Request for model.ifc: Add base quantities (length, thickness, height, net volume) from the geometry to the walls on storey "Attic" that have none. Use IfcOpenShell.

First a look at what the model holds.

```python
import ifcopenshell
import ifcopenshell.util.element
import ifcopenshell.util.unit

model = ifcopenshell.open("model.ifc")
print(model.schema)
for unit_type in ("LENGTHUNIT", "AREAUNIT", "VOLUMEUNIT"):
    print(unit_type, ifcopenshell.util.unit.calculate_unit_scale(model, unit_type))
storey = next(s for s in model.by_type("IfcBuildingStorey") if s.Name == "Attic")
walls = [e for e in ifcopenshell.util.element.get_decomposition(storey) if e.is_a("IfcWall")]
for e in sorted(walls, key=lambda e: e.id()):
    print(e.id(), e.is_a(), e.Name, list(ifcopenshell.util.element.get_psets(e, qtos_only=True)), sep=" | ")
```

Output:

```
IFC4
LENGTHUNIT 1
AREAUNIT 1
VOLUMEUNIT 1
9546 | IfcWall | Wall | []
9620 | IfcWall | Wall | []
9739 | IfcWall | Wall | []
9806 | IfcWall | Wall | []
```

```python
import ifcopenshell
import ifcopenshell.api.pset
import ifcopenshell.geom
import ifcopenshell.util.element
import ifcopenshell.util.shape
import ifcopenshell.util.unit

model = ifcopenshell.open("model.ifc")
unit_scale = ifcopenshell.util.unit.calculate_unit_scale(model)
volume_scale = ifcopenshell.util.unit.calculate_unit_scale(model, "VOLUMEUNIT")
settings = ifcopenshell.geom.settings()

storey = next(s for s in model.by_type("IfcBuildingStorey") if s.Name == "Attic")
walls = [e for e in ifcopenshell.util.element.get_decomposition(storey) if e.is_a("IfcWall")]

for e in sorted(walls, key=lambda e: e.id()):
    if ifcopenshell.util.element.get_psets(e, qtos_only=True, should_inherit=False):
        continue
    # Geometry comes back in metres, in the element's own axes.
    shape = ifcopenshell.geom.create_shape(settings, e)
    values = {
        "Length": ifcopenshell.util.shape.get_x(shape.geometry) / unit_scale,
        "Width": ifcopenshell.util.shape.get_y(shape.geometry) / unit_scale,
        "Height": ifcopenshell.util.shape.get_z(shape.geometry) / unit_scale,
        "NetVolume": ifcopenshell.util.shape.get_volume(shape.geometry) / volume_scale,
    }
    qto = ifcopenshell.api.pset.add_qto(model, product=e, name="Qto_WallBaseQuantities")
    ifcopenshell.api.pset.edit_qto(model, qto=qto, properties=values)
    print(e.id(), {k: round(v, 3) for k, v in values.items()})

model.write("model-out.ifc")
```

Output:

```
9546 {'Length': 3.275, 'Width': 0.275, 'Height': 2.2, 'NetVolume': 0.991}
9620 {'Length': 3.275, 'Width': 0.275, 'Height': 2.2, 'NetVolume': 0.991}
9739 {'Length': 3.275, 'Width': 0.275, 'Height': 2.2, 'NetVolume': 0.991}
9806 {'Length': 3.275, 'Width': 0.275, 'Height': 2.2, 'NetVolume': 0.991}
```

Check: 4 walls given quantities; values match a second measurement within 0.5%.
